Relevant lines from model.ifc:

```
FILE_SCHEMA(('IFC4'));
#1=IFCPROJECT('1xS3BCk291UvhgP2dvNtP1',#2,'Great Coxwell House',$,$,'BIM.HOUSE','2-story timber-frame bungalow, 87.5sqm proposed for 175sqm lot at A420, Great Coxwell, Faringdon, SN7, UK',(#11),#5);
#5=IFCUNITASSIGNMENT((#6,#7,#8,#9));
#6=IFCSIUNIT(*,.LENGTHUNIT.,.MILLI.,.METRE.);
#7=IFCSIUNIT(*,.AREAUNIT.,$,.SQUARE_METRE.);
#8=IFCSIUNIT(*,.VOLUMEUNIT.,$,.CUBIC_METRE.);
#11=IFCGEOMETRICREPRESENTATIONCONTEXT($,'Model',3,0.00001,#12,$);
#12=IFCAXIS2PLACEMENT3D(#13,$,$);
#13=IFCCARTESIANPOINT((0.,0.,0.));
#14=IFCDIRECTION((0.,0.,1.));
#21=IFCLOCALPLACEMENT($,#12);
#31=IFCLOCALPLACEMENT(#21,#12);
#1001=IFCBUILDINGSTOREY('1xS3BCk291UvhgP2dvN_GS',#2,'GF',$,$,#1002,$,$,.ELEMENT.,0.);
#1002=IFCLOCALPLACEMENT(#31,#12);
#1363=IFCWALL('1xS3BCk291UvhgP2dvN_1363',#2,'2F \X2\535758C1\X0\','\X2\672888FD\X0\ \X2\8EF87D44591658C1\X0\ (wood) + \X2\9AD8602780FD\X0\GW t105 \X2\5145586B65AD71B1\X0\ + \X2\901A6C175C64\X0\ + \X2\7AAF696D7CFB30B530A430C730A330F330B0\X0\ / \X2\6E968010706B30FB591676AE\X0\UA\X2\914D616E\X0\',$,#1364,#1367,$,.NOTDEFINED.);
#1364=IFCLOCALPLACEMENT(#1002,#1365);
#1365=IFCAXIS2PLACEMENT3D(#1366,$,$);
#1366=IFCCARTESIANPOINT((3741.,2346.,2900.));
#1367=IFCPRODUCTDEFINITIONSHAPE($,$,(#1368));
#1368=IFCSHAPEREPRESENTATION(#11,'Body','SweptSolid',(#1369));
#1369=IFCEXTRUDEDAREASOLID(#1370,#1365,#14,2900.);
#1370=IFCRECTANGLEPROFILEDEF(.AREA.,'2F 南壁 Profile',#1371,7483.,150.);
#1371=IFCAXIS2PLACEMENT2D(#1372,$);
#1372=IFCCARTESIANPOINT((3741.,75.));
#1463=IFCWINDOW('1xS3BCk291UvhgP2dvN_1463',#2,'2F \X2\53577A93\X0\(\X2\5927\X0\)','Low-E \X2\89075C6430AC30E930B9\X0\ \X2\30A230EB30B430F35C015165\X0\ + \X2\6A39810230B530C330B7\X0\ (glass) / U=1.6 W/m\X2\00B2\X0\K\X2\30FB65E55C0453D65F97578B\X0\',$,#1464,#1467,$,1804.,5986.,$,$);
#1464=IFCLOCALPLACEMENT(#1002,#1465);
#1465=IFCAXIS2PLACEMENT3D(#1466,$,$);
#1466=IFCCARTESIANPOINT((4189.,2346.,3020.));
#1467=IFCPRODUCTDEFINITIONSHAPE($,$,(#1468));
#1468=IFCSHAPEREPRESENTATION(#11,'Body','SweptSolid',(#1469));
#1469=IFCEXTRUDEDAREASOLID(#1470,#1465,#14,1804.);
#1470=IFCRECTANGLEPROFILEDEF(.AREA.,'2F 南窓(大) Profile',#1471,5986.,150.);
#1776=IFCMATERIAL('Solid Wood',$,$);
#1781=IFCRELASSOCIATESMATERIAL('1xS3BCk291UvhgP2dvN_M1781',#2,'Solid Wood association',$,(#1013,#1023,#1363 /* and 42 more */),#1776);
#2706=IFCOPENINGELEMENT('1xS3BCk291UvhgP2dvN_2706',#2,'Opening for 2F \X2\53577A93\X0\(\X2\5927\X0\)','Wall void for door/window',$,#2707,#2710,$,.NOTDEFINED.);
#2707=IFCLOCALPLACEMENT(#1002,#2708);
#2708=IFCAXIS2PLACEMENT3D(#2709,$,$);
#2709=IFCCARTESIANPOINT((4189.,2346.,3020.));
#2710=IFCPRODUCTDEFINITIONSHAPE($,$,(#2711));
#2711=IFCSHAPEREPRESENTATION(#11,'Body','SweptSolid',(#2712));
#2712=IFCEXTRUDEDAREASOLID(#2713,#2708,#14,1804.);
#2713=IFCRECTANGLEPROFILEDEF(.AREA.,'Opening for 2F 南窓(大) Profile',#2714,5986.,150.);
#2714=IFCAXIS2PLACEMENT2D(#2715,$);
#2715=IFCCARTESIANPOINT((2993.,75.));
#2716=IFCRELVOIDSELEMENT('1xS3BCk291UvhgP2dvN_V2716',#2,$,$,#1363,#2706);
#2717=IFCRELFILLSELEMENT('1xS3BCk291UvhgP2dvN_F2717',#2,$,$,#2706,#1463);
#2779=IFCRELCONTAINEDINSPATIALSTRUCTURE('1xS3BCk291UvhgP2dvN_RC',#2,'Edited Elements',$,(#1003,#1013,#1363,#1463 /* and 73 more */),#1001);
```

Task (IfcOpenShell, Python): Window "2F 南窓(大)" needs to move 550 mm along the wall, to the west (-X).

```python
import ifcopenshell
import ifcopenshell.api.geometry
import ifcopenshell.util.placement

model = ifcopenshell.open("model.ifc")

window = model.by_guid("1xS3BCk291UvhgP2dvN_1463")
opening = window.FillsVoids[0].RelatingOpeningElement
wall = opening.VoidsElements[0].RelatingBuildingElement

wall_matrix = ifcopenshell.util.placement.get_local_placement(wall.ObjectPlacement)
shift = wall_matrix[:3, 0] * -550.0
before = ifcopenshell.util.placement.get_local_placement(window.ObjectPlacement)[:3, 3].copy()

# The window is not placed relative to its opening, so move both.
for product in (opening, window):
    matrix = ifcopenshell.util.placement.get_local_placement(product.ObjectPlacement)
    matrix[:3, 3] += shift
    ifcopenshell.api.geometry.edit_object_placement(model, product=product, matrix=matrix, is_si=False)

after = ifcopenshell.util.placement.get_local_placement(window.ObjectPlacement)[:3, 3]
print("window moved by", (after - before).round(3) + 0.0)

model.write("model_updated.ifc")
```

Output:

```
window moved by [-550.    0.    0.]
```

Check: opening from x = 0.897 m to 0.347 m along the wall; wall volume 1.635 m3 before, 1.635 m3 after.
